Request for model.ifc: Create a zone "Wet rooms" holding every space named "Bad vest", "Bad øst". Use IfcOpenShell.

First a look at what the model holds.

```python
import ifcopenshell

model = ifcopenshell.open("model.ifc")
print(model.schema)
seen = {}
for space in model.by_type("IfcSpace"):
    seen[space.LongName] = seen.get(space.LongName, 0) + 1
for name, count in sorted(seen.items(), key=str):
    print(count, "x", name)
print("zones:", [z.Name for z in model.by_type("IfcZone")][:20])
```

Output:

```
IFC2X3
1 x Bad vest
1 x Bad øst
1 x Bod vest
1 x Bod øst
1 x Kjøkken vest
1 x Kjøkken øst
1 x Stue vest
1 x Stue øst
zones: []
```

```python
import ifcopenshell
import ifcopenshell.api.group
import ifcopenshell.api.root

model = ifcopenshell.open("model.ifc")

names = {"Bad vest", "Bad øst"}
spaces = [s for s in model.by_type("IfcSpace") if s.LongName in names]

zone = ifcopenshell.api.root.create_entity(model, ifc_class="IfcZone", name="Wet rooms")
ifcopenshell.api.group.assign_group(model, products=spaces, group=zone)
print(len(spaces), "spaces in", zone.Name)

model.write("model-out.ifc")
```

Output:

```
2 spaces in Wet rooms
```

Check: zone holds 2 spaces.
